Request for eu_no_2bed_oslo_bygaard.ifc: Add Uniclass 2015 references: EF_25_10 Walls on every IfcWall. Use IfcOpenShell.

First a look at what the model holds.

```python
import ifcopenshell

model = ifcopenshell.open("eu_no_2bed_oslo_bygaard.ifc")
print(model.schema)
print("classifications:", [c.Name for c in model.by_type("IfcClassification")])
for ifc_class in ("IfcDoor", "IfcRoof", "IfcStair", "IfcWall", "IfcWindow"):
    print(ifc_class, len(model.by_type(ifc_class)))
```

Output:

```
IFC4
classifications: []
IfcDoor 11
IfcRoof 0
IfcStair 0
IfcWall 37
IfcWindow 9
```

```python
import ifcopenshell
import ifcopenshell.api.classification

model = ifcopenshell.open("eu_no_2bed_oslo_bygaard.ifc")

system = ifcopenshell.api.classification.add_classification(model, classification="Uniclass 2015")

codes = {
    "IfcWall": ("EF_25_10", "Walls"),
}
for ifc_class, (code, name) in codes.items():
    products = model.by_type(ifc_class)
    ifcopenshell.api.classification.add_reference(
        model, products=products, classification=system, identification=code, name=name
    )
    print(code, len(products))

model.write("eu_no_2bed_oslo_bygaard_edited.ifc")
```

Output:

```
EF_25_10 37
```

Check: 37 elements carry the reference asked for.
